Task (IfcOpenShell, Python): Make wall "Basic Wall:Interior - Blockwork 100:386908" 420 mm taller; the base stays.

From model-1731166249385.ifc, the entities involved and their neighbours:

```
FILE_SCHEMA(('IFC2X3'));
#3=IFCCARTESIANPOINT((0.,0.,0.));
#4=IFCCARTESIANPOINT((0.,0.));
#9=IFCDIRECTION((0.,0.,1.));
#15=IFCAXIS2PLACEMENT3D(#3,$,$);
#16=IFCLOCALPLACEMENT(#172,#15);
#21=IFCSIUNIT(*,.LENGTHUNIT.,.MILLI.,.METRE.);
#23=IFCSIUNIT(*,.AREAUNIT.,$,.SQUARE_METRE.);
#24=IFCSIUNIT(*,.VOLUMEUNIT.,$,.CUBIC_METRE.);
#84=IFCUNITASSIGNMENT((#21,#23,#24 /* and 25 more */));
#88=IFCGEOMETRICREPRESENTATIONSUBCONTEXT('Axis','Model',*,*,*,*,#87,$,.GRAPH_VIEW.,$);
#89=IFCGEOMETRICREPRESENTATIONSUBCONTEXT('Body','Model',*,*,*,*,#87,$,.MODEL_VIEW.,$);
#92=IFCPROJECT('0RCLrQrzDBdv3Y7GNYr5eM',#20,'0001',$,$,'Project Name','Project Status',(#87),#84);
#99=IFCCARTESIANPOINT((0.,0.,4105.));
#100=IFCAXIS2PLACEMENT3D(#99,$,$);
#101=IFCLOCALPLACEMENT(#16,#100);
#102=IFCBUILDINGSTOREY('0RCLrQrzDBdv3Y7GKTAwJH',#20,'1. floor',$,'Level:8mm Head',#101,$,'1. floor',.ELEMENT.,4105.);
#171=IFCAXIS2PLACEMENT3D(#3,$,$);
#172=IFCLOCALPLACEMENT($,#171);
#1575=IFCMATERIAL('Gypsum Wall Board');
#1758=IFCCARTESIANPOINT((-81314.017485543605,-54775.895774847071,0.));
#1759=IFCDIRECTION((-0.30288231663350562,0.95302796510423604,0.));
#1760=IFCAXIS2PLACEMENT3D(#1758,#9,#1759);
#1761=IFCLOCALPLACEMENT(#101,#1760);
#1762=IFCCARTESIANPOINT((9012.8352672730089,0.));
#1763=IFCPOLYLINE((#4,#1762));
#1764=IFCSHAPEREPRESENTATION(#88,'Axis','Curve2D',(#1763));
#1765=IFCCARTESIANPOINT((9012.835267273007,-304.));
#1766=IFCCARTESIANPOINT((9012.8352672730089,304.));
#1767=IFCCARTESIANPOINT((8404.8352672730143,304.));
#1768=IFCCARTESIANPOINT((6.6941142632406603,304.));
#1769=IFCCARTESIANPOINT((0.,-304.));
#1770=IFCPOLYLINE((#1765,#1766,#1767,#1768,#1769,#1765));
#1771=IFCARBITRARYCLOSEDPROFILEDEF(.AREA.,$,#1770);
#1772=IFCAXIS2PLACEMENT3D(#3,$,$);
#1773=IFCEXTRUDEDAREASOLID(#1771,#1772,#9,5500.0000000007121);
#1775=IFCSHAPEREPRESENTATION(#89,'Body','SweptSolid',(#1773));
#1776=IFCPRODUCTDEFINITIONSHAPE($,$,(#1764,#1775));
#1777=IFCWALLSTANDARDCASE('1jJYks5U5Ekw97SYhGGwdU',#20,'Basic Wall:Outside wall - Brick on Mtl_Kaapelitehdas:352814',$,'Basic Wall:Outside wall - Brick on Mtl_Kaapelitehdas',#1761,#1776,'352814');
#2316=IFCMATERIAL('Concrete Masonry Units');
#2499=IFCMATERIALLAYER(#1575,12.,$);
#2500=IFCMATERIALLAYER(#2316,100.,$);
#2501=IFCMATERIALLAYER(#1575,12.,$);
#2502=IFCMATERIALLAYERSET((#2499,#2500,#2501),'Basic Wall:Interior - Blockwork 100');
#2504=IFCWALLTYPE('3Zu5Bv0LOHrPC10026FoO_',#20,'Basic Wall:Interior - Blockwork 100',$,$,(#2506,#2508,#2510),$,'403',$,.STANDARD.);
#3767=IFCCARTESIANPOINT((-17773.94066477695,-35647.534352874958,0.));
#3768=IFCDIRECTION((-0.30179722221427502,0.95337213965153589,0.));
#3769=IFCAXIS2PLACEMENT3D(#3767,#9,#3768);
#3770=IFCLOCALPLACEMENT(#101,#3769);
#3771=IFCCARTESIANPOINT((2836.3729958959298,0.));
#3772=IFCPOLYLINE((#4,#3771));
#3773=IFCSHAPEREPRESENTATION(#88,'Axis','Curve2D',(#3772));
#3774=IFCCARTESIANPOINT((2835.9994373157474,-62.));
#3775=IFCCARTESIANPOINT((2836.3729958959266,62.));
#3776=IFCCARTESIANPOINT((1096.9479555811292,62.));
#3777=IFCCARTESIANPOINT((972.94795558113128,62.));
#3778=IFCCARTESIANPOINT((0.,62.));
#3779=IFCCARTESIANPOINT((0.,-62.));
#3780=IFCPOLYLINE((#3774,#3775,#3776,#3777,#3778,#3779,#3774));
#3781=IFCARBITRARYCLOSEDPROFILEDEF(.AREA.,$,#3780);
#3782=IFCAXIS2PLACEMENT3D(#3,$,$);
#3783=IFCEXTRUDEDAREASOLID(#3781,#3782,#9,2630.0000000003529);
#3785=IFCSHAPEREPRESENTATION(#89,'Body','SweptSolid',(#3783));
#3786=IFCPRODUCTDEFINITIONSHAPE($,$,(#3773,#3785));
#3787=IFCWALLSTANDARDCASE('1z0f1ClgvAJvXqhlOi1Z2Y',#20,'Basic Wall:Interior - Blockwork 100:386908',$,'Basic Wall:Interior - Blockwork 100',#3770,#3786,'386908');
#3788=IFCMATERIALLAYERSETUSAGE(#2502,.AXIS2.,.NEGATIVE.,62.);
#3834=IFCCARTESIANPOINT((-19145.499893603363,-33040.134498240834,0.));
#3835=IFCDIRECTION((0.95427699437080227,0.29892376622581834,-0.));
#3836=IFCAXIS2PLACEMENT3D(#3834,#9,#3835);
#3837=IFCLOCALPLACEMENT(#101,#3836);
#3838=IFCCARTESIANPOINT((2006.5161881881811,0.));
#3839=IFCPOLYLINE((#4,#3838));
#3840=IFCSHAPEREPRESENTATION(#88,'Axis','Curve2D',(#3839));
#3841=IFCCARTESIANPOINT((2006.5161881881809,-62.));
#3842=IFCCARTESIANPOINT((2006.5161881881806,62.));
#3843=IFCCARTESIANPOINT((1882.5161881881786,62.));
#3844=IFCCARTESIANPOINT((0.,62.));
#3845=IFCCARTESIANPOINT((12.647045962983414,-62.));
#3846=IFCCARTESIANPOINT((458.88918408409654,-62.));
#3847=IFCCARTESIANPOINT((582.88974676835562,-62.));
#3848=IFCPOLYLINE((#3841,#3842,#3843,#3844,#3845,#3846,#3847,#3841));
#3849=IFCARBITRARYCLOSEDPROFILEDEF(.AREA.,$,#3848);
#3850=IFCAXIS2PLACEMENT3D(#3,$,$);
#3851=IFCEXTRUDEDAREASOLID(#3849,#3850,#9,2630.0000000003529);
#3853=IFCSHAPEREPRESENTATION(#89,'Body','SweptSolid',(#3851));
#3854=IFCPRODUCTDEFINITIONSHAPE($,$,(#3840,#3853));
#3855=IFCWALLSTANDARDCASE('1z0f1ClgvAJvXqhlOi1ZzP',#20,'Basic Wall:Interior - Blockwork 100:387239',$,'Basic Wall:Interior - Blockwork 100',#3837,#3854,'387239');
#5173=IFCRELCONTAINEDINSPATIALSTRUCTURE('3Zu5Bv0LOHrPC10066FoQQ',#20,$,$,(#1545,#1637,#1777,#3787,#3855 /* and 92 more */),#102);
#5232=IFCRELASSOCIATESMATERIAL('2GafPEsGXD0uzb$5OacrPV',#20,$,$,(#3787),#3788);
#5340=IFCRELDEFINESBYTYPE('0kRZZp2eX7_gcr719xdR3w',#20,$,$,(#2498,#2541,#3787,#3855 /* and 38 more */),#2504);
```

```python
import ifcopenshell
import ifcopenshell.geom
import ifcopenshell.util.representation
import ifcopenshell.util.shape
import ifcopenshell.util.unit

model = ifcopenshell.open("model-1731166249385.ifc")
unit_scale = ifcopenshell.util.unit.calculate_unit_scale(model)
settings = ifcopenshell.geom.settings()


def volume(element):
    """Net volume in cubic metres, openings subtracted."""
    shape = ifcopenshell.geom.create_shape(settings, element)
    return ifcopenshell.util.shape.get_volume(shape.geometry)


wall = model.by_guid("1z0f1ClgvAJvXqhlOi1Z2Y")
before = volume(wall)

body = ifcopenshell.util.representation.get_representation(wall, "Model", "Body")
solid = body.Items[0]
old_height = solid.Depth
solid.Depth += 0.42 / unit_scale
after = volume(wall)

print(f"height {old_height:g} -> {solid.Depth:g}, volume {before:.3f} -> {after:.3f} m3")

model.write("model-1731166249385_v2.ifc")
```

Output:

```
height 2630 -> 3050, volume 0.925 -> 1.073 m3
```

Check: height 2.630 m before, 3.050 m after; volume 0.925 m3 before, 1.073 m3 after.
